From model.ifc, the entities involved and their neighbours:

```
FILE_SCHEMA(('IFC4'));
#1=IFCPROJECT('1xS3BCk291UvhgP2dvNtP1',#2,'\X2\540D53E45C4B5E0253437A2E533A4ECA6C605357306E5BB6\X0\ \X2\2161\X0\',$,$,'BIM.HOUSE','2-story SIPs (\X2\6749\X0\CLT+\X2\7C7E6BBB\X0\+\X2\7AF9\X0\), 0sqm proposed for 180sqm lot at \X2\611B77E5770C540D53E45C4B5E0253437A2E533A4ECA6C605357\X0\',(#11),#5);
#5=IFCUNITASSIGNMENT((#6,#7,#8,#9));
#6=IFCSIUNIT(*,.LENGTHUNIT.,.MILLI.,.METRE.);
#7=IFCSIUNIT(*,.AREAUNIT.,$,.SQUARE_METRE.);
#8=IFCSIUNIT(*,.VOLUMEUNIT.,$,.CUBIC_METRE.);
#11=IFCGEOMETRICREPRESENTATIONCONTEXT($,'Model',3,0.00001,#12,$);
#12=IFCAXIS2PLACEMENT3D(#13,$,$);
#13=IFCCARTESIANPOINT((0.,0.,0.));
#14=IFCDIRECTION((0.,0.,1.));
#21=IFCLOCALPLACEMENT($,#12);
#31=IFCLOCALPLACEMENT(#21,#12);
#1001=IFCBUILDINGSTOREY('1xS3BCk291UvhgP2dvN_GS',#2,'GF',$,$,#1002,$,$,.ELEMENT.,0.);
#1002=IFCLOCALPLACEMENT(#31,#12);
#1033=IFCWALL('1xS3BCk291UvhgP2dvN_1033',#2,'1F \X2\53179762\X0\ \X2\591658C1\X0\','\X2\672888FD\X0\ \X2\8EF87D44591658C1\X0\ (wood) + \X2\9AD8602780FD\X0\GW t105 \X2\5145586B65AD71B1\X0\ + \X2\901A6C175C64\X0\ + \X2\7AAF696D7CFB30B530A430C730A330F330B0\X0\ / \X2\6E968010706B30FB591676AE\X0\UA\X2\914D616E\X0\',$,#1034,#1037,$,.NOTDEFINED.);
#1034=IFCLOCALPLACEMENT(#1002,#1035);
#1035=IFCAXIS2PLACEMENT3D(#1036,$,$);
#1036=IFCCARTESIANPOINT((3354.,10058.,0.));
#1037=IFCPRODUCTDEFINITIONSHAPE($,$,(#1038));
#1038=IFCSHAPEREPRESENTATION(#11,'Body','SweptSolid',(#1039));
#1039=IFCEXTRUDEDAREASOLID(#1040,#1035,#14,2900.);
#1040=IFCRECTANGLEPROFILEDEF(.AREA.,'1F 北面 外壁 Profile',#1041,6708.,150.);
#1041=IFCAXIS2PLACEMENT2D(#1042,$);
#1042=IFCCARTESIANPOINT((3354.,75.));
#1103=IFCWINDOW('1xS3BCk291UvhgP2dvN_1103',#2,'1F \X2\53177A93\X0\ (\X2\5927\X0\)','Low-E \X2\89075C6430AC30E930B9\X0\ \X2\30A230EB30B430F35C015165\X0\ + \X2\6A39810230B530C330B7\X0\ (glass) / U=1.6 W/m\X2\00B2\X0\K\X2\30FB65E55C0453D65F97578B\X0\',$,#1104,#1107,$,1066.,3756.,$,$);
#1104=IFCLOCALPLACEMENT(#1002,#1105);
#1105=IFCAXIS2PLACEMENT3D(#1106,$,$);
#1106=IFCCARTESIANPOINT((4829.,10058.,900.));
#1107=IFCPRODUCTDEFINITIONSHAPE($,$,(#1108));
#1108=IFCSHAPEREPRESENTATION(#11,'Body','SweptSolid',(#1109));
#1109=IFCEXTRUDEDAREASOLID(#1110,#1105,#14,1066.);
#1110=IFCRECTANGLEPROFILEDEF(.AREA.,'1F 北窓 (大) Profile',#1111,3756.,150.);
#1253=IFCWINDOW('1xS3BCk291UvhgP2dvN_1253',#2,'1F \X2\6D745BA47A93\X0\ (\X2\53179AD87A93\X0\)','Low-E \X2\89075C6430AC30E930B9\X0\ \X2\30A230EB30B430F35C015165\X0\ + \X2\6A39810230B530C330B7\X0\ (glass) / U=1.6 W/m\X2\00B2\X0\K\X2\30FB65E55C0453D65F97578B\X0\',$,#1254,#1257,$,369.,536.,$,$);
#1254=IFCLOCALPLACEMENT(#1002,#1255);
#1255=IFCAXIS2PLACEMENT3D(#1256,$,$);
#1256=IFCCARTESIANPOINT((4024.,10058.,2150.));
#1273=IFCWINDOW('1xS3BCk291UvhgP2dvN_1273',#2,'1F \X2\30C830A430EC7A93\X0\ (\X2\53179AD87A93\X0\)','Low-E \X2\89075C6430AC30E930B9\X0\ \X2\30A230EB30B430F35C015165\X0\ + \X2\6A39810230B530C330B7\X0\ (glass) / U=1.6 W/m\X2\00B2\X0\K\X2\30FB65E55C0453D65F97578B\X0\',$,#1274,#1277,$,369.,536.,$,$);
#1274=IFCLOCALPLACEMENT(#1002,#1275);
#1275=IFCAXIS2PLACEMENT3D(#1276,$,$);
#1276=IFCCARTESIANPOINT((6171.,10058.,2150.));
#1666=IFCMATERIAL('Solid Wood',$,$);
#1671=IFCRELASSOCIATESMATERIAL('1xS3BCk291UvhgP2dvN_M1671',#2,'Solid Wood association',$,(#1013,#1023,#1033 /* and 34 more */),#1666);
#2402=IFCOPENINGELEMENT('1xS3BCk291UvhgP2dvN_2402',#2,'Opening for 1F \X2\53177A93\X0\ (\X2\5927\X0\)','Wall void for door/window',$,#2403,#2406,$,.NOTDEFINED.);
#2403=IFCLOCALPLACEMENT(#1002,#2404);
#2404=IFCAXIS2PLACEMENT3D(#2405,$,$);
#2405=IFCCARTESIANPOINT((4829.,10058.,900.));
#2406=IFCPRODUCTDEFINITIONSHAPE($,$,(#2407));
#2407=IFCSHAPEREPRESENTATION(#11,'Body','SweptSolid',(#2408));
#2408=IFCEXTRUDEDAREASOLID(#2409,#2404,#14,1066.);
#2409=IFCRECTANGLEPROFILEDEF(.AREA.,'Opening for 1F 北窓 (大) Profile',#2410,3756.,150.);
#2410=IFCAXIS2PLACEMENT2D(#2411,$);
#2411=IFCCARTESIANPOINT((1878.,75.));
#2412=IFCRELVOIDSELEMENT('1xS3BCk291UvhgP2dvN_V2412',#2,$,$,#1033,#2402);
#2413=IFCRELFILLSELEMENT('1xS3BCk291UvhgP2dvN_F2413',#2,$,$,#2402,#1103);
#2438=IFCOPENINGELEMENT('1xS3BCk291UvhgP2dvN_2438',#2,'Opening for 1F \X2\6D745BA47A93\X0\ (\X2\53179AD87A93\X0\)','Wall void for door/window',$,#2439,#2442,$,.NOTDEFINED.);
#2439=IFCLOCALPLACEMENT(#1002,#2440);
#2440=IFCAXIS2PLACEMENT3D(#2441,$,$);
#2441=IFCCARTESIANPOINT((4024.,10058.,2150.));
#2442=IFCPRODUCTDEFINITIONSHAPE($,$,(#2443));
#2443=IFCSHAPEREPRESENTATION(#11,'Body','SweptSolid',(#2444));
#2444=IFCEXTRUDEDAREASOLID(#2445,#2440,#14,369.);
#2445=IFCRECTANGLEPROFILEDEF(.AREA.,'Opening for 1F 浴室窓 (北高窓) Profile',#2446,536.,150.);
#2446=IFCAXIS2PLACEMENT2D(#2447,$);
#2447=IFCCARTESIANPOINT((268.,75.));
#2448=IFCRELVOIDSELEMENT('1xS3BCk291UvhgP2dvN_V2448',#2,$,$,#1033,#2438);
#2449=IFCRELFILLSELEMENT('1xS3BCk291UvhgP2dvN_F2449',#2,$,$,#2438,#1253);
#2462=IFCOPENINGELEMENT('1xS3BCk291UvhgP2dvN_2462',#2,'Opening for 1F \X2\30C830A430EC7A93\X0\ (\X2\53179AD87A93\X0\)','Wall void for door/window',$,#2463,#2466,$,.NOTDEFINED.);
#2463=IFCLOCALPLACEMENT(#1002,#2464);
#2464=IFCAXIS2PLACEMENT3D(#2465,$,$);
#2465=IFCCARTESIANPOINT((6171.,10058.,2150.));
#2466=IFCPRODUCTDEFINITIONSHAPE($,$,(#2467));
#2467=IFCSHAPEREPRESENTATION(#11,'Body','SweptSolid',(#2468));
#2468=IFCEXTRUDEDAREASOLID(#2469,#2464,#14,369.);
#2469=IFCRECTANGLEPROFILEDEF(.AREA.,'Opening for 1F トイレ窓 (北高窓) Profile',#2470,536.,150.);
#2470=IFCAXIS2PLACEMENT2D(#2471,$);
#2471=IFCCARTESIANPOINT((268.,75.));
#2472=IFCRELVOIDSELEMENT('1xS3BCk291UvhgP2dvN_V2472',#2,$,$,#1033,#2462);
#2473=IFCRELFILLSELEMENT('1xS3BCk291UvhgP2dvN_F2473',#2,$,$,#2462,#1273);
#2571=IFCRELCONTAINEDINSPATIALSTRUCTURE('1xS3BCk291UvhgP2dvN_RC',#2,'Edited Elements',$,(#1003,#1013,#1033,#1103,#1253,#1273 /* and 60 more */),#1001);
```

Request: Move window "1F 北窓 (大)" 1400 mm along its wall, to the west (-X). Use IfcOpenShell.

```python
import ifcopenshell
import ifcopenshell.api.geometry
import ifcopenshell.util.placement
import ifcopenshell.util.unit

model = ifcopenshell.open("model.ifc")
unit_scale = ifcopenshell.util.unit.calculate_unit_scale(model)

window = model.by_id(1103)
opening = window.FillsVoids[0].RelatingOpeningElement
wall = opening.VoidsElements[0].RelatingBuildingElement

wall_matrix = ifcopenshell.util.placement.get_local_placement(wall.ObjectPlacement)
shift = wall_matrix[:3, 0] * -1.4 / unit_scale
before = ifcopenshell.util.placement.get_local_placement(window.ObjectPlacement)[:3, 3].copy()

# The window is not placed relative to its opening, so move both.
for product in (opening, window):
    matrix = ifcopenshell.util.placement.get_local_placement(product.ObjectPlacement)
    matrix[:3, 3] += shift
    ifcopenshell.api.geometry.edit_object_placement(model, product=product, matrix=matrix, is_si=False)

after = ifcopenshell.util.placement.get_local_placement(window.ObjectPlacement)[:3, 3]
print("window moved by", (after - before).round(3) + 0.0)

model.write("model_updated.ifc")
```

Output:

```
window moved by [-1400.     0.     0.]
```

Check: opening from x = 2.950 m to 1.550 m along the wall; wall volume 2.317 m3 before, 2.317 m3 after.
